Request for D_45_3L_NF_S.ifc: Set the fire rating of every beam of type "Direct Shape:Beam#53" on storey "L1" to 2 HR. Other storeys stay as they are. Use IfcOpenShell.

First a look at what the model holds.

```python
import ifcopenshell
import ifcopenshell.util.element

model = ifcopenshell.open("D_45_3L_NF_S.ifc")
print(model.schema)
storey = next(s for s in model.by_type("IfcBuildingStorey") if s.Name == "L1")
beams = [e for e in ifcopenshell.util.element.get_decomposition(storey) if e.is_a("IfcBeam")]
seen = {}
for e in beams:
    element_type = ifcopenshell.util.element.get_type(e)
    key = (element_type.Name if element_type != e and element_type else None, ifcopenshell.util.element.get_pset(e, "Pset_BeamCommon", "FireRating"))
    seen[key] = seen.get(key, 0) + 1
for (name, value), count in sorted(seen.items(), key=str):
    print(count, "x", name, "|", value)
```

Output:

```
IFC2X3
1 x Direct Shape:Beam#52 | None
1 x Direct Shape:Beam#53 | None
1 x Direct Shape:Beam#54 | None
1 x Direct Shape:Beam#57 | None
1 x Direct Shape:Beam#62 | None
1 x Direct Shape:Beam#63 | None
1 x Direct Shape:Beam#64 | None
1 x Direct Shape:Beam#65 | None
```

```python
import ifcopenshell
import ifcopenshell.api.pset
import ifcopenshell.util.element

model = ifcopenshell.open("D_45_3L_NF_S.ifc")

storey = next(s for s in model.by_type("IfcBuildingStorey") if s.Name == "L1")
beams = [e for e in ifcopenshell.util.element.get_decomposition(storey) if e.is_a("IfcBeam")]

count = 0
for e in beams:
    element_type = ifcopenshell.util.element.get_type(e)
    if element_type in (None, e) or element_type.Name != "Direct Shape:Beam#53":
        continue
    # add_pset returns the element's existing set when there is one.
    pset = ifcopenshell.api.pset.add_pset(model, product=e, name="Pset_BeamCommon")
    ifcopenshell.api.pset.edit_pset(model, pset=pset, properties={"FireRating": "2 HR"})
    count += 1

print(count, "beams updated")

model.write("D_45_3L_NF_S_v2.ifc")
```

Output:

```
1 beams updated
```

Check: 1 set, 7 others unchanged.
